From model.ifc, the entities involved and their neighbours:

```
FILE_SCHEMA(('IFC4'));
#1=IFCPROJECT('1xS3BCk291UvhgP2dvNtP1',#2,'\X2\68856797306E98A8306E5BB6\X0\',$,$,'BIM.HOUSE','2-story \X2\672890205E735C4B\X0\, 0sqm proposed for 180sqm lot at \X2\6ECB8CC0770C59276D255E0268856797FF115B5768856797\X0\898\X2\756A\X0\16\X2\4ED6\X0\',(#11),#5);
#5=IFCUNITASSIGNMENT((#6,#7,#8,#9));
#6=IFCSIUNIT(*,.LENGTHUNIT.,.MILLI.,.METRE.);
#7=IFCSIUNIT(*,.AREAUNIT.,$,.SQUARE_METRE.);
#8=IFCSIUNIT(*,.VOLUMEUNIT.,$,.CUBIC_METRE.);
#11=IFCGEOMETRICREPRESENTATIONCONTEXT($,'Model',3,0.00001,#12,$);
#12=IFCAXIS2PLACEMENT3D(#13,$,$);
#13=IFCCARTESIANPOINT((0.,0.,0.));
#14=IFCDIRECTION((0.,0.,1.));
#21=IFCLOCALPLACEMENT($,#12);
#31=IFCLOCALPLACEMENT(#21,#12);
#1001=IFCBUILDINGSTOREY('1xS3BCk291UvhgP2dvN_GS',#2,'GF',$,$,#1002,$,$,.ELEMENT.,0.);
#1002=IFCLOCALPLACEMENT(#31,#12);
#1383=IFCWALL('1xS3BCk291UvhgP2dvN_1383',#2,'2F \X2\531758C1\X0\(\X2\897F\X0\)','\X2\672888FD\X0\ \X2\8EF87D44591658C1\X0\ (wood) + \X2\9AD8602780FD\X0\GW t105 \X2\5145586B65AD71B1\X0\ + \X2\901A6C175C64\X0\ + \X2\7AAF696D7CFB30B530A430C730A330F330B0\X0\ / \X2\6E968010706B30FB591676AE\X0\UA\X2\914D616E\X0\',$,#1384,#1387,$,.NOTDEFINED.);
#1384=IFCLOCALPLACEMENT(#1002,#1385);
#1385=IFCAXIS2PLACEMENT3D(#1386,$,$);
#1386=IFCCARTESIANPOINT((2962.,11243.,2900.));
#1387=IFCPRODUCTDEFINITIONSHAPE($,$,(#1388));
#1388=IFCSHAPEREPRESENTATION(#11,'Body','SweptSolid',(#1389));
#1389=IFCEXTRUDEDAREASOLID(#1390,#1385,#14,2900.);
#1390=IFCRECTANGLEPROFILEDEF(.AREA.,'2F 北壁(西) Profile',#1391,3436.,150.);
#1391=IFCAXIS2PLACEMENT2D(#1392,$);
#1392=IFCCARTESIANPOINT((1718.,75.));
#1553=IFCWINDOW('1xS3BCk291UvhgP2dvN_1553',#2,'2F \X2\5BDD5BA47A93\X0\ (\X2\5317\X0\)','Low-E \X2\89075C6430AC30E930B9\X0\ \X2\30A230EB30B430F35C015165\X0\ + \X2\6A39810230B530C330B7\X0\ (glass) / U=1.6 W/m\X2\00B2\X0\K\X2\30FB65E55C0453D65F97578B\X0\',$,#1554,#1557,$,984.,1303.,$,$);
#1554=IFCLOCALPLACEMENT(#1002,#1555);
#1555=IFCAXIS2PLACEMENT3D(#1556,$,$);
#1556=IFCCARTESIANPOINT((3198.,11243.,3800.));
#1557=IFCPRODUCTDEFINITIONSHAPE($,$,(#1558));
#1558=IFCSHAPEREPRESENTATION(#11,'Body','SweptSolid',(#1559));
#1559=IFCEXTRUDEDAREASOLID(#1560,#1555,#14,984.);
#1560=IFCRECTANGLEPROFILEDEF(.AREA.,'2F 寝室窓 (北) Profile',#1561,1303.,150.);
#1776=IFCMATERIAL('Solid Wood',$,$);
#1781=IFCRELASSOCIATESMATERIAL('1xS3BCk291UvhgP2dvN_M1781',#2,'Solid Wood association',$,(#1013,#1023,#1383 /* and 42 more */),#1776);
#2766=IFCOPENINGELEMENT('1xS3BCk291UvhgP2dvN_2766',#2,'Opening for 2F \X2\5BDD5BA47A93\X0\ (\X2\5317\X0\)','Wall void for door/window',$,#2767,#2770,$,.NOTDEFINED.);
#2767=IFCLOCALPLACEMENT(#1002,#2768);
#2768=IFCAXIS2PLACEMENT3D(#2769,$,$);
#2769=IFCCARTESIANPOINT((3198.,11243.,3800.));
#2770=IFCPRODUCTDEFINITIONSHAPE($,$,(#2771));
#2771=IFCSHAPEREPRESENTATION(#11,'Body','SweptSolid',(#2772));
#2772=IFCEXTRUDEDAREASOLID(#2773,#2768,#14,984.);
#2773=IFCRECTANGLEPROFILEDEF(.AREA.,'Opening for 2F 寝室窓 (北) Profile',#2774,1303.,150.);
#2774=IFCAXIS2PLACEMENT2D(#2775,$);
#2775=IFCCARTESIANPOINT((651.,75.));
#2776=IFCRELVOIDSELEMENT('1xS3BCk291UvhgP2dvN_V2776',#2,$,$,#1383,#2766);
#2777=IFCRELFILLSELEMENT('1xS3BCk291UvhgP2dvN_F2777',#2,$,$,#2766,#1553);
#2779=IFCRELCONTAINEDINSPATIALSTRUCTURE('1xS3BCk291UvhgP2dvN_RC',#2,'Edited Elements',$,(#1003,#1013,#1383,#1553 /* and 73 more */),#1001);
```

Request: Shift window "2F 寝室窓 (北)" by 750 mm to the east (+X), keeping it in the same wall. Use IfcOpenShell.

```python
import ifcopenshell
import ifcopenshell.api.geometry
import ifcopenshell.util.placement

model = ifcopenshell.open("model.ifc")

window = model.by_guid("1xS3BCk291UvhgP2dvN_1553")
opening = window.FillsVoids[0].RelatingOpeningElement
wall = opening.VoidsElements[0].RelatingBuildingElement

wall_matrix = ifcopenshell.util.placement.get_local_placement(wall.ObjectPlacement)
shift = wall_matrix[:3, 0] * 750.0
before = ifcopenshell.util.placement.get_local_placement(window.ObjectPlacement)[:3, 3].copy()

# The window is not placed relative to its opening, so move both.
for product in (opening, window):
    matrix = ifcopenshell.util.placement.get_local_placement(product.ObjectPlacement)
    matrix[:3, 3] += shift
    ifcopenshell.api.geometry.edit_object_placement(model, product=product, matrix=matrix, is_si=False)

after = ifcopenshell.util.placement.get_local_placement(window.ObjectPlacement)[:3, 3]
print("window moved by", (after - before).round(3) + 0.0)

model.write("model-out.ifc")
```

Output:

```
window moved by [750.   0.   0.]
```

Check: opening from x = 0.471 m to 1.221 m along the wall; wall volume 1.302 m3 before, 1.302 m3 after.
